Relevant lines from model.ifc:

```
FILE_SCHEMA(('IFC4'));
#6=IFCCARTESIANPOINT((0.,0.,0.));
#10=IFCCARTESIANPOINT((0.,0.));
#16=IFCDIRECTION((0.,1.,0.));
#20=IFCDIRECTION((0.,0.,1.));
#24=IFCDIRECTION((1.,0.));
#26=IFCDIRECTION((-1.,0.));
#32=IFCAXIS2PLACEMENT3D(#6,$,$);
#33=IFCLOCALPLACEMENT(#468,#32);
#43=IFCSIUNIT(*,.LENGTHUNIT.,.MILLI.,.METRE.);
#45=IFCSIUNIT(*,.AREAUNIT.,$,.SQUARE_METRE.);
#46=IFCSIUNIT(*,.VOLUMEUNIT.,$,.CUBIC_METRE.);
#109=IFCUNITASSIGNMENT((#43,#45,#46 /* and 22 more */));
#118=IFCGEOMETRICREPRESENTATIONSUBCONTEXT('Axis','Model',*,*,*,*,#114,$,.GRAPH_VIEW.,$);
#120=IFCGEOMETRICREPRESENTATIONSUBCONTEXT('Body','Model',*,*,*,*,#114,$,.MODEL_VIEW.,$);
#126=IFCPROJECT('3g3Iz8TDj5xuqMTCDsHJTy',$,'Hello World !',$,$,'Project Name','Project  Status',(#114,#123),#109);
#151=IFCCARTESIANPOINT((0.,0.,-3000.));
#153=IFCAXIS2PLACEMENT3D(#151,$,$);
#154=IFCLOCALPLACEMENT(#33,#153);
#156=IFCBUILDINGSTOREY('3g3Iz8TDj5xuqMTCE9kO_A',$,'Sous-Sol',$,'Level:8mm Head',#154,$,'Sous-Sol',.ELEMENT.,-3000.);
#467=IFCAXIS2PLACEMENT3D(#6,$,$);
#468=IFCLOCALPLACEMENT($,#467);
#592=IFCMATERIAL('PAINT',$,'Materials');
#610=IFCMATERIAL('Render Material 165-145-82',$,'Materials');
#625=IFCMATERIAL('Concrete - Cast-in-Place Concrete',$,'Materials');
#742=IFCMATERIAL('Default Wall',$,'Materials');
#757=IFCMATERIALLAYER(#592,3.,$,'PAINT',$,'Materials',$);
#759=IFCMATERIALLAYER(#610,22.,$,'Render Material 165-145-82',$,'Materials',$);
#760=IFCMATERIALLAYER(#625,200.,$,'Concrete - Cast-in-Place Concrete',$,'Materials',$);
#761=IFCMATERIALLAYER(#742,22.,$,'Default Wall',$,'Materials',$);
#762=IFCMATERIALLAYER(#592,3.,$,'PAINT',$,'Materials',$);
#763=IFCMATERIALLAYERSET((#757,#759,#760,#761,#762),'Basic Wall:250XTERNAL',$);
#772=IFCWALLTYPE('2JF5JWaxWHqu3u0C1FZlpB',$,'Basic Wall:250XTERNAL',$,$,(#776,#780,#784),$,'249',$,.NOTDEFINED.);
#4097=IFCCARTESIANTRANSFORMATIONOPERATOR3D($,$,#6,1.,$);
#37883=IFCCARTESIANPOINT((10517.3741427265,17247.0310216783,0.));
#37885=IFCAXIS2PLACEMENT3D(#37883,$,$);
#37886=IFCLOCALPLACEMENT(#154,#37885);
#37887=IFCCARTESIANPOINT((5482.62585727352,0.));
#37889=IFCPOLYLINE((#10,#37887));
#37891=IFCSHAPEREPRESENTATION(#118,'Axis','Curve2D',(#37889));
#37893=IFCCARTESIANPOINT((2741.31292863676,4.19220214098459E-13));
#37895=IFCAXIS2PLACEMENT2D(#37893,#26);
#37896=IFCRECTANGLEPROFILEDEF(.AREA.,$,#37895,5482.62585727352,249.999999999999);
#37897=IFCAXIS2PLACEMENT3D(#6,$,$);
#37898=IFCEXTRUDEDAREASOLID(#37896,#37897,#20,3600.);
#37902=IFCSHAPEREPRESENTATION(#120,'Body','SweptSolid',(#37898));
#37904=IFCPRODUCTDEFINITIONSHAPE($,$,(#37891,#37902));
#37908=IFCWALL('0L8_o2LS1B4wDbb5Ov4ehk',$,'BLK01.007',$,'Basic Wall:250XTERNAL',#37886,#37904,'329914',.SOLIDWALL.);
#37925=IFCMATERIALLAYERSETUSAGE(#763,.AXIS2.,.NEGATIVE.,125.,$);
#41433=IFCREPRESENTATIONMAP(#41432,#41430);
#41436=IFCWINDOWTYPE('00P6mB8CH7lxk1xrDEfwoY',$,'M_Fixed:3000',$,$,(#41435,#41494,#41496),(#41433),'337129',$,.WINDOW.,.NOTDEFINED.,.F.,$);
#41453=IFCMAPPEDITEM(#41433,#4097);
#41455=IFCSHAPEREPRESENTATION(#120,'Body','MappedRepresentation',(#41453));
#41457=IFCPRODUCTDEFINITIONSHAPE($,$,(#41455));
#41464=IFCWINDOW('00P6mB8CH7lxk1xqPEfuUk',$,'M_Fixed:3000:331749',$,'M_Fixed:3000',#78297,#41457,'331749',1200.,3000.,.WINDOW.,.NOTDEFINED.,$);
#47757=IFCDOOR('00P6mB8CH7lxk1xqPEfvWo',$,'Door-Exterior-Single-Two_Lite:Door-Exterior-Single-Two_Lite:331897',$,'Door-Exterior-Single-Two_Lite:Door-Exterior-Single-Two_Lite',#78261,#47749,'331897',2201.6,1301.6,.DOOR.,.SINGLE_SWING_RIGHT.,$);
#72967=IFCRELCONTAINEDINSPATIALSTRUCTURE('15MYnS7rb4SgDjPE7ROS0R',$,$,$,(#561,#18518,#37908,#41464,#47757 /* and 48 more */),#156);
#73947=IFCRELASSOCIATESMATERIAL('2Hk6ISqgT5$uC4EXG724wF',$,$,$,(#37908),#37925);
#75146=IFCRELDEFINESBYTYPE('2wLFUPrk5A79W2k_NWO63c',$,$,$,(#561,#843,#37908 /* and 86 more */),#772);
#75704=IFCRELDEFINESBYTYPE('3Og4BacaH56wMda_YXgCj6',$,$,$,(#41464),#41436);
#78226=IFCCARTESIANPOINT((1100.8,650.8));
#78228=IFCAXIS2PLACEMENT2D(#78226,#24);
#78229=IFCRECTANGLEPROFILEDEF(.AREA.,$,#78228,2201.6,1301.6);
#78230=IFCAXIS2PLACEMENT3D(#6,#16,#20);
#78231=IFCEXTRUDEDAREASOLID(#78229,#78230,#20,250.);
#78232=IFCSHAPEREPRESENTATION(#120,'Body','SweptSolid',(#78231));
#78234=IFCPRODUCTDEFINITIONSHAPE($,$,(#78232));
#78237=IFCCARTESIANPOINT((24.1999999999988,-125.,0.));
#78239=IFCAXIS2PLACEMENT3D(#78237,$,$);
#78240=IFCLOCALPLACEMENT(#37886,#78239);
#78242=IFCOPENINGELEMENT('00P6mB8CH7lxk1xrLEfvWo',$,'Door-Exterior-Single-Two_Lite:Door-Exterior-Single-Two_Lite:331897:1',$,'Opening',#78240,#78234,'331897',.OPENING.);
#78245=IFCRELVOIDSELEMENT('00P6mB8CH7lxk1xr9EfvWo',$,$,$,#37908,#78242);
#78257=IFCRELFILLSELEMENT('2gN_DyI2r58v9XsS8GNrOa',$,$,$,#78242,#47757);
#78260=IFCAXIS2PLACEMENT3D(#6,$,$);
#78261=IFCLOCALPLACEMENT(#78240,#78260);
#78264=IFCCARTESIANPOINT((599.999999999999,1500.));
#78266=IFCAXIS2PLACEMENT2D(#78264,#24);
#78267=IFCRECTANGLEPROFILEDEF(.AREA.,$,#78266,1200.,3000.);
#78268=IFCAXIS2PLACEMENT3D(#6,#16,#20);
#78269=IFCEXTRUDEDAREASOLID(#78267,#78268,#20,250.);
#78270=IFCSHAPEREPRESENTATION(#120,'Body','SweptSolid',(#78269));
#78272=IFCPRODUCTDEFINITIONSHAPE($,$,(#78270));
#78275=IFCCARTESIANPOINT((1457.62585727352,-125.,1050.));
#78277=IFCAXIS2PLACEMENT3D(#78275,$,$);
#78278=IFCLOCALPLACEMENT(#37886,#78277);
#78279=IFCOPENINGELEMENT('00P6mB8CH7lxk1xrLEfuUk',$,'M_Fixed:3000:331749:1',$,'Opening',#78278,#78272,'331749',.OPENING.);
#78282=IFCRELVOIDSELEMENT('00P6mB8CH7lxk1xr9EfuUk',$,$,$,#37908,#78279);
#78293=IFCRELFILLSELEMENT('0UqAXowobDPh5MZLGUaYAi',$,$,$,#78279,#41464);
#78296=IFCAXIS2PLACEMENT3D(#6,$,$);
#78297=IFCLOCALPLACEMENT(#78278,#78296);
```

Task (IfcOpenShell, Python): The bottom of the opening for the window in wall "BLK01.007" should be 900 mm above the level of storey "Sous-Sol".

```python
import numpy as np
import ifcopenshell
import ifcopenshell.api.geometry
import ifcopenshell.geom
import ifcopenshell.util.element
import ifcopenshell.util.placement
import ifcopenshell.util.shape
import ifcopenshell.util.unit

model = ifcopenshell.open("model.ifc")
unit_scale = ifcopenshell.util.unit.calculate_unit_scale(model)

window = model.by_guid("00P6mB8CH7lxk1xqPEfuUk")
opening = window.FillsVoids[0].RelatingOpeningElement
storey = ifcopenshell.util.element.get_container(window, ifc_class="IfcBuildingStorey")
level = ifcopenshell.util.placement.get_local_placement(storey.ObjectPlacement)[2, 3]

# The opening's origin need not be at the sill, so measure its lowest point.
shape = ifcopenshell.geom.create_shape(ifcopenshell.geom.settings(), opening)
bottom = ifcopenshell.util.shape.get_shape_bottom_elevation(shape, shape.geometry) / unit_scale
dz = level + 900.0 - bottom

shift = np.array([0.0, 0.0, dz])
# The window is placed relative to its opening, so it follows when the opening moves.
matrix = ifcopenshell.util.placement.get_local_placement(opening.ObjectPlacement)
matrix[:3, 3] += shift
ifcopenshell.api.geometry.edit_object_placement(
    model, product=opening, matrix=matrix, is_si=False, should_transform_children=True
)

print(f"moved by {dz * unit_scale:+.3f} m")

model.write("model_updated.ifc")
```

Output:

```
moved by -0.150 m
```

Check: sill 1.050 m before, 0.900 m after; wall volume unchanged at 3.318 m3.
